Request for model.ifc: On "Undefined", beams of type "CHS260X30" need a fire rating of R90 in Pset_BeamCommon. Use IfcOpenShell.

First a look at what the model holds.

```python
import ifcopenshell
import ifcopenshell.util.element

model = ifcopenshell.open("model.ifc")
print(model.schema)
storey = next(s for s in model.by_type("IfcBuildingStorey") if s.Name == "Undefined")
beams = [e for e in ifcopenshell.util.element.get_decomposition(storey) if e.is_a("IfcBeam")]
seen = {}
for e in beams:
    element_type = ifcopenshell.util.element.get_type(e)
    key = (element_type.Name if element_type != e and element_type else None, ifcopenshell.util.element.get_pset(e, "Pset_BeamCommon", "FireRating"))
    seen[key] = seen.get(key, 0) + 1
for (name, value), count in sorted(seen.items(), key=str):
    print(count, "x", name, "|", value)
```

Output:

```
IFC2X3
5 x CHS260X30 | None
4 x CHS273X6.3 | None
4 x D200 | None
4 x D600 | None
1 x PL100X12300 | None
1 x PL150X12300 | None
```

```python
import ifcopenshell
import ifcopenshell.api.pset
import ifcopenshell.util.element

model = ifcopenshell.open("model.ifc")

storey = next(s for s in model.by_type("IfcBuildingStorey") if s.Name == "Undefined")
beams = [e for e in ifcopenshell.util.element.get_decomposition(storey) if e.is_a("IfcBeam")]

count = 0
for e in beams:
    element_type = ifcopenshell.util.element.get_type(e)
    if element_type in (None, e) or element_type.Name != "CHS260X30":
        continue
    found = ifcopenshell.util.element.get_pset(e, "Pset_BeamCommon", should_inherit=False)
    if found:
        pset = model.by_id(found["id"])
        if len(ifcopenshell.util.element.get_elements_by_pset(pset)) > 1:
            pset = ifcopenshell.api.pset.unshare_pset(model, products=[e], pset=pset)[0]
    else:
        pset = ifcopenshell.api.pset.add_pset(model, product=e, name="Pset_BeamCommon")
    ifcopenshell.api.pset.edit_pset(model, pset=pset, properties={"FireRating": "R90"})
    count += 1

print(count, "beams updated")

model.write("model_updated.ifc")
```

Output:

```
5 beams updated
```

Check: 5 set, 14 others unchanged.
